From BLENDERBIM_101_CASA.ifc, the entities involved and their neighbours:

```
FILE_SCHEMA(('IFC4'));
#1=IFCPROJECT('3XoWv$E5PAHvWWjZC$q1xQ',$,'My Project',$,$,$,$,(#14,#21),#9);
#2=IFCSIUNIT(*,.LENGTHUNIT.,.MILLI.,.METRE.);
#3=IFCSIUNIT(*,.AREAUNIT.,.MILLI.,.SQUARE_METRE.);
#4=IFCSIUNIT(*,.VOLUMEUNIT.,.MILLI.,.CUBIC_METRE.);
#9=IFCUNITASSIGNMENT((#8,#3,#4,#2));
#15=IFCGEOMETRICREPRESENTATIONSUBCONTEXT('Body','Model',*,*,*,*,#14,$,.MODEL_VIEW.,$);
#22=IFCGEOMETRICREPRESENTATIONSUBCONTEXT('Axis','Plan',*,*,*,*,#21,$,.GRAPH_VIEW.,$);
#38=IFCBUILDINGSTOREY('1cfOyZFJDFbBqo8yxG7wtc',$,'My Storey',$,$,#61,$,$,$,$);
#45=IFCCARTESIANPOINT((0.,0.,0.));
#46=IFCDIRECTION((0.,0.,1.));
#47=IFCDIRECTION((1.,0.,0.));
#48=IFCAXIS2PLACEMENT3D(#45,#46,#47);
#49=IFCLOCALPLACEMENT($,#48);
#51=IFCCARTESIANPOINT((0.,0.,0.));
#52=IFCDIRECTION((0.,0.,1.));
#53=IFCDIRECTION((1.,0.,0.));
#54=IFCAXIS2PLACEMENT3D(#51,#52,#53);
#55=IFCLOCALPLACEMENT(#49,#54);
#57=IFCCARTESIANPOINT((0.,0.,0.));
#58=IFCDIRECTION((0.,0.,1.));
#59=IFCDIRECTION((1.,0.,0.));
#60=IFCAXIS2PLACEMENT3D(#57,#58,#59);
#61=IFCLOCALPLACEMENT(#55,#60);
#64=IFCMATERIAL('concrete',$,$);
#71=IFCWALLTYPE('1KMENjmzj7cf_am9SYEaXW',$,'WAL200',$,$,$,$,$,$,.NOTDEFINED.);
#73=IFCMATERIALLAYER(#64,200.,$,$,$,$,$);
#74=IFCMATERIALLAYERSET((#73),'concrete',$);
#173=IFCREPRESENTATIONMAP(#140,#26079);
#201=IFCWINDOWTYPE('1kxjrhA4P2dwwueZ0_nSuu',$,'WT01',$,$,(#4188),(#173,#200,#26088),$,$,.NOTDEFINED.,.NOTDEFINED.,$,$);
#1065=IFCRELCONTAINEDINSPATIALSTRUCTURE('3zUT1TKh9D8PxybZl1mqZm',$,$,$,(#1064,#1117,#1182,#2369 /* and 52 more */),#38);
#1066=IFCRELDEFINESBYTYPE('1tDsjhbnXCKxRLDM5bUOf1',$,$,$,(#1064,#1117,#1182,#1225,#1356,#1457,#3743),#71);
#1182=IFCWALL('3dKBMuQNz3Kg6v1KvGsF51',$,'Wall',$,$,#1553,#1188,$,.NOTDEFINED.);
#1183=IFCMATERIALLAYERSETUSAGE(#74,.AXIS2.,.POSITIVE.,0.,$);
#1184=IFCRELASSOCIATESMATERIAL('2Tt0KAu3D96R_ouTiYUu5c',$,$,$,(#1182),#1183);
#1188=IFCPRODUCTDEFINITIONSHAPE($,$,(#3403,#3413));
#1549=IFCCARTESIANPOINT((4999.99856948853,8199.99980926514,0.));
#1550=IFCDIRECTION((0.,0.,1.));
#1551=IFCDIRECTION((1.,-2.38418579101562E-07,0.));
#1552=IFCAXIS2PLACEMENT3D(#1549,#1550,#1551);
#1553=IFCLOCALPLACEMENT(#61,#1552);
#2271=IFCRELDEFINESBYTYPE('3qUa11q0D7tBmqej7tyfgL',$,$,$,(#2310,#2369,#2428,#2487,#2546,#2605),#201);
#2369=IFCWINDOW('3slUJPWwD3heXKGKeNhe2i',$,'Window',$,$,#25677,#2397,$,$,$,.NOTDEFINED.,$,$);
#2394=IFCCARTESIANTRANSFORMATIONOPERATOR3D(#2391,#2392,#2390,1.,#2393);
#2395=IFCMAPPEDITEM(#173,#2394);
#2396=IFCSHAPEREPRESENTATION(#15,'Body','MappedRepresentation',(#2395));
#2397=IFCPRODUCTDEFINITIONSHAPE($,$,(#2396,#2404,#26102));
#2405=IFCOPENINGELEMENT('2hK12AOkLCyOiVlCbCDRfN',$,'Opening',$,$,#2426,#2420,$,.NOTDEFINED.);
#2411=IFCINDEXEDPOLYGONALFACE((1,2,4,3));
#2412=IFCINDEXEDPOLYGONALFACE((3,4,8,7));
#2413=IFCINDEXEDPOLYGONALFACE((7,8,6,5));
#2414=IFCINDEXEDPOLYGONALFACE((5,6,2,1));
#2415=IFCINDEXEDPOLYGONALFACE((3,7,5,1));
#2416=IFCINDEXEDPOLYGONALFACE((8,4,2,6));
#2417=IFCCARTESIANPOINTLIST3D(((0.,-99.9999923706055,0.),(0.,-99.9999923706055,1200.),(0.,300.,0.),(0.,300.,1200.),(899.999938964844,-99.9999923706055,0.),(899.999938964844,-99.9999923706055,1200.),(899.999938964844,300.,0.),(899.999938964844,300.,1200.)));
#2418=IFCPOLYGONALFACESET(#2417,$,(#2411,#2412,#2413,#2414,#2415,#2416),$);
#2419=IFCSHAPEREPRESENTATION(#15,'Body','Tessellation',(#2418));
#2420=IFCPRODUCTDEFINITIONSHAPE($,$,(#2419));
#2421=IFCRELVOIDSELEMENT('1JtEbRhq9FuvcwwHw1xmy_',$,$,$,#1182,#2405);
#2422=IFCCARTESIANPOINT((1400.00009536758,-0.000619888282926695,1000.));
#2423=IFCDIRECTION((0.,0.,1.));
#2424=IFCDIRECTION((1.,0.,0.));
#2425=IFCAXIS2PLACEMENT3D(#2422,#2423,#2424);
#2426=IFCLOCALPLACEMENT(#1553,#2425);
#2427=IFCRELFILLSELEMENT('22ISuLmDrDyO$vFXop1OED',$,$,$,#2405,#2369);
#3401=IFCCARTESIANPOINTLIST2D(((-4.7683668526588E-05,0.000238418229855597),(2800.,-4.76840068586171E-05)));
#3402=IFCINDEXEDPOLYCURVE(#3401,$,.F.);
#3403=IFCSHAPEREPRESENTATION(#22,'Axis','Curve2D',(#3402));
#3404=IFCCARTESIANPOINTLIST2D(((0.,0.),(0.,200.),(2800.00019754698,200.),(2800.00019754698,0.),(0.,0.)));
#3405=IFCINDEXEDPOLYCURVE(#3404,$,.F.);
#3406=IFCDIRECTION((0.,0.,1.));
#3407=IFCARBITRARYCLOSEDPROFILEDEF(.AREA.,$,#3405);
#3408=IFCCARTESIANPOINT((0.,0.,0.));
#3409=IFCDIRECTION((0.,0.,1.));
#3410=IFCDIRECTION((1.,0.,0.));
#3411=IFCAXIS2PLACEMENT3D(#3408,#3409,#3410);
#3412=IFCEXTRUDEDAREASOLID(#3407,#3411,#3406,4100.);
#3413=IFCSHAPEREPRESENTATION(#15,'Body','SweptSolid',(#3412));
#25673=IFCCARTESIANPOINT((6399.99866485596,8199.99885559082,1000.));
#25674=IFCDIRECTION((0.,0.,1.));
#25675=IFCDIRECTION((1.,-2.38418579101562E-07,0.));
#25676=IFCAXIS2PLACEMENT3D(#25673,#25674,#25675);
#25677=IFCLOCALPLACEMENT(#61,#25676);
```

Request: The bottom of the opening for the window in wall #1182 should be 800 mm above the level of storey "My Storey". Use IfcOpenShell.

```python
import numpy as np
import ifcopenshell
import ifcopenshell.api.geometry
import ifcopenshell.geom
import ifcopenshell.util.element
import ifcopenshell.util.placement
import ifcopenshell.util.shape
import ifcopenshell.util.unit

model = ifcopenshell.open("BLENDERBIM_101_CASA.ifc")
unit_scale = ifcopenshell.util.unit.calculate_unit_scale(model)

window = model.by_guid("3slUJPWwD3heXKGKeNhe2i")
opening = window.FillsVoids[0].RelatingOpeningElement
storey = ifcopenshell.util.element.get_container(window, ifc_class="IfcBuildingStorey")
level = ifcopenshell.util.placement.get_local_placement(storey.ObjectPlacement)[2, 3]

# The opening's origin need not be at the sill, so measure its lowest point.
shape = ifcopenshell.geom.create_shape(ifcopenshell.geom.settings(), opening)
bottom = ifcopenshell.util.shape.get_shape_bottom_elevation(shape, shape.geometry) / unit_scale
dz = level + 0.8 / unit_scale - bottom

shift = np.array([0.0, 0.0, dz])
# The window is not placed relative to its opening, so move both.
for product in (opening, window):
    matrix = ifcopenshell.util.placement.get_local_placement(product.ObjectPlacement)
    matrix[:3, 3] += shift
    ifcopenshell.api.geometry.edit_object_placement(model, product=product, matrix=matrix, is_si=False)

print(f"moved by {dz * unit_scale:+.3f} m")

model.write("BLENDERBIM_101_CASA_rev.ifc")
```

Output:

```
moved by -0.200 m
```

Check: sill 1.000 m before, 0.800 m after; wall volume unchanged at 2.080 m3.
